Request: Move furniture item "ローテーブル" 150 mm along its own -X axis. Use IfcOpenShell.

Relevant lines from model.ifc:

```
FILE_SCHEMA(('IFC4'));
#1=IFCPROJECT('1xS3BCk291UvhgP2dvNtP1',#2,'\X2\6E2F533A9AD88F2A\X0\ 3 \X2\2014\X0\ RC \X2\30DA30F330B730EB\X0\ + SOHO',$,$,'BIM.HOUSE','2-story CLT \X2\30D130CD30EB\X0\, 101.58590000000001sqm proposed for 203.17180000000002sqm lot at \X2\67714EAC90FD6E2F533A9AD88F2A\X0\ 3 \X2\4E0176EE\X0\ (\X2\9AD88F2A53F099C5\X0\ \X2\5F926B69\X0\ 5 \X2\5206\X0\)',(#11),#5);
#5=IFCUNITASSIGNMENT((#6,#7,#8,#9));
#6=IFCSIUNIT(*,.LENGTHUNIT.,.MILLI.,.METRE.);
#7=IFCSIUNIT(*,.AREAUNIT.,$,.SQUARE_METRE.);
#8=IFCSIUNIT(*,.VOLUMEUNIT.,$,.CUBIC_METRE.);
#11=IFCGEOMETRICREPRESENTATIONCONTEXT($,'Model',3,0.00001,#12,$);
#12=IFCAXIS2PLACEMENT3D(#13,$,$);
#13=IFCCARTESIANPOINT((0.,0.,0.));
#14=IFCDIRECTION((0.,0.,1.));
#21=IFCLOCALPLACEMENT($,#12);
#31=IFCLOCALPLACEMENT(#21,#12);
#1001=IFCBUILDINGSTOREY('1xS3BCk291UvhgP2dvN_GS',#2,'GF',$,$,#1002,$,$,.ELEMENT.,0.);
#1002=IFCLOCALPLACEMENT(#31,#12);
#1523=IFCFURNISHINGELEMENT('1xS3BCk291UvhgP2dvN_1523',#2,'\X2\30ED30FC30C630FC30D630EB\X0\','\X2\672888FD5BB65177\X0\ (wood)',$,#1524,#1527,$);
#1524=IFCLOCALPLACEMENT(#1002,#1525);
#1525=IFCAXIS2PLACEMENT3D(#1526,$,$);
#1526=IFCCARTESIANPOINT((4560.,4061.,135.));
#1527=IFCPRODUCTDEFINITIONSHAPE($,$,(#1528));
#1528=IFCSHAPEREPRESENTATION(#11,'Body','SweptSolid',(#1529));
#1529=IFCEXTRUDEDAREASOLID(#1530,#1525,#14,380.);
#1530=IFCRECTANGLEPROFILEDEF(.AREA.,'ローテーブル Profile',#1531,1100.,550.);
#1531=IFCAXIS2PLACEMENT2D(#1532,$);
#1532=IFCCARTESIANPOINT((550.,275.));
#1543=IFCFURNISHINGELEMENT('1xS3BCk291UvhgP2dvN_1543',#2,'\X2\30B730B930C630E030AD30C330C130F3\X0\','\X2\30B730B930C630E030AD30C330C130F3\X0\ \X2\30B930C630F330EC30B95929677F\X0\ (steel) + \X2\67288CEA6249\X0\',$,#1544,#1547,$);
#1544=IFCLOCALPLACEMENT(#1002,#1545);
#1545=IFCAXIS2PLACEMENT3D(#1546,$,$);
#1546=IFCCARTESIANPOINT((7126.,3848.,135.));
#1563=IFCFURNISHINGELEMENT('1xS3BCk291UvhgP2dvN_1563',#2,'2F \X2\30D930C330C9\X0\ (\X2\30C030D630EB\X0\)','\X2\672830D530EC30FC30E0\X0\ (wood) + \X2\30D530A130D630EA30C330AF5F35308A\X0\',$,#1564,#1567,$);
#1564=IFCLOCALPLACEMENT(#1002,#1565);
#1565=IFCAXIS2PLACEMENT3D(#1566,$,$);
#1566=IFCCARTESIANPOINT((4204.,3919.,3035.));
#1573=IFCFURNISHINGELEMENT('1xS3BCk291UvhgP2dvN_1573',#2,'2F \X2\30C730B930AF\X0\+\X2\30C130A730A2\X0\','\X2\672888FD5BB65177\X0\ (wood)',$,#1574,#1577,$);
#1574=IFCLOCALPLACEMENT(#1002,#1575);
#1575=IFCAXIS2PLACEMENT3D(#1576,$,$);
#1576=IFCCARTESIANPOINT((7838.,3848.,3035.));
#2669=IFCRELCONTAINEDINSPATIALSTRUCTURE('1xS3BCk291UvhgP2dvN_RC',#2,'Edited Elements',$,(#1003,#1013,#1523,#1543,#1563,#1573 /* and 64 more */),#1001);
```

```python
import ifcopenshell
import ifcopenshell.api.geometry
import ifcopenshell.util.placement
import ifcopenshell.util.unit

model = ifcopenshell.open("model.ifc")
unit_scale = ifcopenshell.util.unit.calculate_unit_scale(model)

item = model.by_guid("1xS3BCk291UvhgP2dvN_1523")
matrix = ifcopenshell.util.placement.get_local_placement(item.ObjectPlacement)
matrix[:3, 3] -= matrix[:3, 0] * 0.15 / unit_scale
ifcopenshell.api.geometry.edit_object_placement(model, product=item, matrix=matrix, is_si=False)

print(ifcopenshell.util.placement.get_local_placement(item.ObjectPlacement).round(3) + 0.0)

model.write("model-out.ifc")
```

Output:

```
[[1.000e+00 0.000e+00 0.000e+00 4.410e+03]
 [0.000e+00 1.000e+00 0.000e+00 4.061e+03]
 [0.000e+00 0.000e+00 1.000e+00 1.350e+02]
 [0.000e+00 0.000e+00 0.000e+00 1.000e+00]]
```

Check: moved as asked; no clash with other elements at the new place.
